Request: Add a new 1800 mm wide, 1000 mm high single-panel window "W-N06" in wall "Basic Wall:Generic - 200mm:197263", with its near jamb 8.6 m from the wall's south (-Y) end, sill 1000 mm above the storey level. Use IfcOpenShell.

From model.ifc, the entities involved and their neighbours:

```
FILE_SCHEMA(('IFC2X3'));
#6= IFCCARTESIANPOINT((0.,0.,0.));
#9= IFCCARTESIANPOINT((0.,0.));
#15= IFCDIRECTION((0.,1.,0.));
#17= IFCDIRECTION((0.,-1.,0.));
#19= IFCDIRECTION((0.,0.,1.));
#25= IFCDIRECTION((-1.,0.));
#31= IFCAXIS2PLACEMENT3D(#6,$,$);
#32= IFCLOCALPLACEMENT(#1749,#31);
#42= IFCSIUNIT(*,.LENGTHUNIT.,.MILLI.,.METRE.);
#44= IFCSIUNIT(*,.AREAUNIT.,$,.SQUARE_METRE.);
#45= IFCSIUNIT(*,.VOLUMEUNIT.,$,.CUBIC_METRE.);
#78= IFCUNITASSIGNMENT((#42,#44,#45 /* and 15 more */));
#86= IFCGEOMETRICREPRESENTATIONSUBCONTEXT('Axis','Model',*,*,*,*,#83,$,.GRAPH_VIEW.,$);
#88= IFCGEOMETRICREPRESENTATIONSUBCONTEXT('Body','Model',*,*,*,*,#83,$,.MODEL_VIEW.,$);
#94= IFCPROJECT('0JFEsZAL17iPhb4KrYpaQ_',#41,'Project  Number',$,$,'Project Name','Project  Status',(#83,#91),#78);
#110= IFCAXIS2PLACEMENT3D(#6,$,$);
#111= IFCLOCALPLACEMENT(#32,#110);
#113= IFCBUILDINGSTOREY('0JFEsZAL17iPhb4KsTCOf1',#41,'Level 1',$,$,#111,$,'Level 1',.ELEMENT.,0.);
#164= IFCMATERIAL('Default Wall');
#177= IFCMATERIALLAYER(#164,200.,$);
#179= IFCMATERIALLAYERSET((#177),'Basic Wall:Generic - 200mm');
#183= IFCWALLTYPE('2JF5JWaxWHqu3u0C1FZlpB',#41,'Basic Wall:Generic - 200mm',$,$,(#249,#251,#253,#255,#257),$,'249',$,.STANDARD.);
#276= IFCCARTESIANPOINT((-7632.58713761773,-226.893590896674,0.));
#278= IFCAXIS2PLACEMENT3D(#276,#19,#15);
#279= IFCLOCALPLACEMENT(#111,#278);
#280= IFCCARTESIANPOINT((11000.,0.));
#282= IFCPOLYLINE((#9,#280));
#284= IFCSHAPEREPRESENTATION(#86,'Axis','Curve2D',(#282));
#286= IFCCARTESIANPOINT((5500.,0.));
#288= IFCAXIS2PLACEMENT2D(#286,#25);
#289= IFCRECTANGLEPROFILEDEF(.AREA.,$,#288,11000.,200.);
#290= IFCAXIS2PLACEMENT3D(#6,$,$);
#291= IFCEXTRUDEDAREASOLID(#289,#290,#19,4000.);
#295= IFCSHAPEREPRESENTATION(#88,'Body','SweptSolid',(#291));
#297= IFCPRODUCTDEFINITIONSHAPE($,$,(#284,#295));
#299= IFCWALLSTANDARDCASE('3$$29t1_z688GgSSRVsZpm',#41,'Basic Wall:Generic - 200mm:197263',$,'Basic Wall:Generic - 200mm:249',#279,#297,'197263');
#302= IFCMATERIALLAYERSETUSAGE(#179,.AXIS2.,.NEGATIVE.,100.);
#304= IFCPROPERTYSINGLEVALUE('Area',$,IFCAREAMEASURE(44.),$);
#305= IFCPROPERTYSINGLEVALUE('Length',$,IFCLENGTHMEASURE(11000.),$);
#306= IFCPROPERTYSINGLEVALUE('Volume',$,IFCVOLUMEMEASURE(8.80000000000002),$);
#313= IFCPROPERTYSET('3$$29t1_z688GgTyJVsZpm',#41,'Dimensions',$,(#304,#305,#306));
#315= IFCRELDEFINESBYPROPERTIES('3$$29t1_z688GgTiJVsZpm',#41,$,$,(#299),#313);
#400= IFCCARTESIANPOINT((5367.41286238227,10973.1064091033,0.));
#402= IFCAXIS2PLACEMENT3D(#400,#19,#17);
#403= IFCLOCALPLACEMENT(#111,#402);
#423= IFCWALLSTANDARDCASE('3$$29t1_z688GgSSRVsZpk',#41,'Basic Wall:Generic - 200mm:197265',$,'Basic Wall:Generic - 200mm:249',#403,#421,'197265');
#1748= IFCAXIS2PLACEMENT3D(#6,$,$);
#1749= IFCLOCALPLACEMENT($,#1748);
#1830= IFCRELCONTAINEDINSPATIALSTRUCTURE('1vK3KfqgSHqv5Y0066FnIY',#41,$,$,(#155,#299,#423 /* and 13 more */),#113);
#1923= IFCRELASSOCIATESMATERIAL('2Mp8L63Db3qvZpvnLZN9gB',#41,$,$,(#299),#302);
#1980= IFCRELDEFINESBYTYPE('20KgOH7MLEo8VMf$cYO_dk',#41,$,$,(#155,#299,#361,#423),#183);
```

```python
import numpy as np
import ifcopenshell
import ifcopenshell.api.feature
import ifcopenshell.api.geometry
import ifcopenshell.api.pset
import ifcopenshell.api.root
import ifcopenshell.api.spatial
import ifcopenshell.api.type
import ifcopenshell.geom
import ifcopenshell.util.element
import ifcopenshell.util.placement
import ifcopenshell.util.representation
import ifcopenshell.util.shape
import ifcopenshell.util.unit

model = ifcopenshell.open("model.ifc")
unit_scale = ifcopenshell.util.unit.calculate_unit_scale(model)
area_scale = ifcopenshell.util.unit.calculate_unit_scale(model, "AREAUNIT")
volume_scale = ifcopenshell.util.unit.calculate_unit_scale(model, "VOLUMEUNIT")
settings = ifcopenshell.geom.settings()


def volume(element):
    """Net volume in cubic metres, openings subtracted."""
    shape = ifcopenshell.geom.create_shape(settings, element)
    return ifcopenshell.util.shape.get_volume(shape.geometry)


wall = model.by_id(299)
storey = ifcopenshell.util.element.get_container(wall, ifc_class="IfcBuildingStorey")
context = ifcopenshell.util.representation.get_context(model, "Model", "Body", "MODEL_VIEW")
before = volume(wall)

width, height, from_end, sill = 1.8, 1, 8.6, 1  # metres

# The wall runs along its own X axis, and the end named is its -X end.
wall_shape = ifcopenshell.geom.create_shape(settings, wall)
x, y, z = ifcopenshell.util.shape.get_vertices(wall_shape.geometry).T
start = x.min() + from_end
face, thickness = float(y.min()), float(y.max() - y.min())
wall_matrix = ifcopenshell.util.placement.get_local_placement(wall.ObjectPlacement)
level = ifcopenshell.util.placement.get_local_placement(storey.ObjectPlacement)[2, 3]


def in_wall(x, y):
    """Placement at x, y metres in the wall's axes, at sill height."""
    matrix = wall_matrix.copy()
    matrix[:, 3] = wall_matrix @ np.array([x / unit_scale, y / unit_scale, 0.0, 1.0])
    matrix[2, 3] = level + sill / unit_scale
    return matrix


# Opening: a box that overshoots both wall faces by 50 mm.
opening = ifcopenshell.api.root.create_entity(model, ifc_class="IfcOpeningElement")
box = ifcopenshell.api.geometry.add_wall_representation(
    model, context=context, length=width, height=height, thickness=thickness + 0.1
)
ifcopenshell.api.geometry.assign_representation(model, product=opening, representation=box)
ifcopenshell.api.geometry.edit_object_placement(model, product=opening, matrix=in_wall(start, face - 0.05), is_si=False)
ifcopenshell.api.feature.add_feature(model, feature=opening, element=wall)

window = ifcopenshell.api.root.create_entity(model, ifc_class="IfcWindow", name="W-N06")
window.OverallWidth, window.OverallHeight = width / unit_scale, height / unit_scale
body = ifcopenshell.api.geometry.add_window_representation(
    model,
    context=context,
    overall_width=window.OverallWidth,
    overall_height=window.OverallHeight,
    partition_type="SINGLE_PANEL",
)
ifcopenshell.api.geometry.assign_representation(model, product=window, representation=body)
ifcopenshell.api.spatial.assign_container(model, products=[window], relating_structure=storey)
fills = ifcopenshell.api.feature.add_filling(model, opening=opening, element=window)
fills.OwnerHistory = window.OwnerHistory  # required in IFC2X3

# IFC2X3 keeps the operation on the window style.
style = ifcopenshell.api.root.create_entity(model, ifc_class="IfcWindowStyle", name="W-N06")
style.OperationType, style.ConstructionType = "SINGLE_PANEL", "NOTDEFINED"
style.ParameterTakesPrecedence = style.Sizeable = False
ifcopenshell.api.type.assign_type(model, related_objects=[window], relating_type=style)

# Centre the window in the wall's thickness.
ifcopenshell.api.geometry.edit_object_placement(model, product=window, matrix=in_wall(start, face), is_si=False)
window_shape = ifcopenshell.geom.create_shape(settings, window)
depth = ifcopenshell.util.shape.get_vertices(window_shape.geometry)[:, 1]
offset = face + thickness / 2 - (depth.min() + depth.max()) / 2
ifcopenshell.api.geometry.edit_object_placement(model, product=window, matrix=in_wall(start, offset), is_si=False)

after = volume(wall)

# Update the wall's stored quantities.
pset = model.by_id(ifcopenshell.util.element.get_pset(wall, "Dimensions", should_inherit=False)["id"])
ifcopenshell.api.pset.edit_pset(model, pset=pset, properties={
    "Area": model.create_entity("IfcAreaMeasure", after / thickness / area_scale),
    "Volume": model.create_entity("IfcVolumeMeasure", after / volume_scale),
})

print(f"wall volume {before:.3f} -> {after:.3f} m3")

model.write("model_v2.ifc")
```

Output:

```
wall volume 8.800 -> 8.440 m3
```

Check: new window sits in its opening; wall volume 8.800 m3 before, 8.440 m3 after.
